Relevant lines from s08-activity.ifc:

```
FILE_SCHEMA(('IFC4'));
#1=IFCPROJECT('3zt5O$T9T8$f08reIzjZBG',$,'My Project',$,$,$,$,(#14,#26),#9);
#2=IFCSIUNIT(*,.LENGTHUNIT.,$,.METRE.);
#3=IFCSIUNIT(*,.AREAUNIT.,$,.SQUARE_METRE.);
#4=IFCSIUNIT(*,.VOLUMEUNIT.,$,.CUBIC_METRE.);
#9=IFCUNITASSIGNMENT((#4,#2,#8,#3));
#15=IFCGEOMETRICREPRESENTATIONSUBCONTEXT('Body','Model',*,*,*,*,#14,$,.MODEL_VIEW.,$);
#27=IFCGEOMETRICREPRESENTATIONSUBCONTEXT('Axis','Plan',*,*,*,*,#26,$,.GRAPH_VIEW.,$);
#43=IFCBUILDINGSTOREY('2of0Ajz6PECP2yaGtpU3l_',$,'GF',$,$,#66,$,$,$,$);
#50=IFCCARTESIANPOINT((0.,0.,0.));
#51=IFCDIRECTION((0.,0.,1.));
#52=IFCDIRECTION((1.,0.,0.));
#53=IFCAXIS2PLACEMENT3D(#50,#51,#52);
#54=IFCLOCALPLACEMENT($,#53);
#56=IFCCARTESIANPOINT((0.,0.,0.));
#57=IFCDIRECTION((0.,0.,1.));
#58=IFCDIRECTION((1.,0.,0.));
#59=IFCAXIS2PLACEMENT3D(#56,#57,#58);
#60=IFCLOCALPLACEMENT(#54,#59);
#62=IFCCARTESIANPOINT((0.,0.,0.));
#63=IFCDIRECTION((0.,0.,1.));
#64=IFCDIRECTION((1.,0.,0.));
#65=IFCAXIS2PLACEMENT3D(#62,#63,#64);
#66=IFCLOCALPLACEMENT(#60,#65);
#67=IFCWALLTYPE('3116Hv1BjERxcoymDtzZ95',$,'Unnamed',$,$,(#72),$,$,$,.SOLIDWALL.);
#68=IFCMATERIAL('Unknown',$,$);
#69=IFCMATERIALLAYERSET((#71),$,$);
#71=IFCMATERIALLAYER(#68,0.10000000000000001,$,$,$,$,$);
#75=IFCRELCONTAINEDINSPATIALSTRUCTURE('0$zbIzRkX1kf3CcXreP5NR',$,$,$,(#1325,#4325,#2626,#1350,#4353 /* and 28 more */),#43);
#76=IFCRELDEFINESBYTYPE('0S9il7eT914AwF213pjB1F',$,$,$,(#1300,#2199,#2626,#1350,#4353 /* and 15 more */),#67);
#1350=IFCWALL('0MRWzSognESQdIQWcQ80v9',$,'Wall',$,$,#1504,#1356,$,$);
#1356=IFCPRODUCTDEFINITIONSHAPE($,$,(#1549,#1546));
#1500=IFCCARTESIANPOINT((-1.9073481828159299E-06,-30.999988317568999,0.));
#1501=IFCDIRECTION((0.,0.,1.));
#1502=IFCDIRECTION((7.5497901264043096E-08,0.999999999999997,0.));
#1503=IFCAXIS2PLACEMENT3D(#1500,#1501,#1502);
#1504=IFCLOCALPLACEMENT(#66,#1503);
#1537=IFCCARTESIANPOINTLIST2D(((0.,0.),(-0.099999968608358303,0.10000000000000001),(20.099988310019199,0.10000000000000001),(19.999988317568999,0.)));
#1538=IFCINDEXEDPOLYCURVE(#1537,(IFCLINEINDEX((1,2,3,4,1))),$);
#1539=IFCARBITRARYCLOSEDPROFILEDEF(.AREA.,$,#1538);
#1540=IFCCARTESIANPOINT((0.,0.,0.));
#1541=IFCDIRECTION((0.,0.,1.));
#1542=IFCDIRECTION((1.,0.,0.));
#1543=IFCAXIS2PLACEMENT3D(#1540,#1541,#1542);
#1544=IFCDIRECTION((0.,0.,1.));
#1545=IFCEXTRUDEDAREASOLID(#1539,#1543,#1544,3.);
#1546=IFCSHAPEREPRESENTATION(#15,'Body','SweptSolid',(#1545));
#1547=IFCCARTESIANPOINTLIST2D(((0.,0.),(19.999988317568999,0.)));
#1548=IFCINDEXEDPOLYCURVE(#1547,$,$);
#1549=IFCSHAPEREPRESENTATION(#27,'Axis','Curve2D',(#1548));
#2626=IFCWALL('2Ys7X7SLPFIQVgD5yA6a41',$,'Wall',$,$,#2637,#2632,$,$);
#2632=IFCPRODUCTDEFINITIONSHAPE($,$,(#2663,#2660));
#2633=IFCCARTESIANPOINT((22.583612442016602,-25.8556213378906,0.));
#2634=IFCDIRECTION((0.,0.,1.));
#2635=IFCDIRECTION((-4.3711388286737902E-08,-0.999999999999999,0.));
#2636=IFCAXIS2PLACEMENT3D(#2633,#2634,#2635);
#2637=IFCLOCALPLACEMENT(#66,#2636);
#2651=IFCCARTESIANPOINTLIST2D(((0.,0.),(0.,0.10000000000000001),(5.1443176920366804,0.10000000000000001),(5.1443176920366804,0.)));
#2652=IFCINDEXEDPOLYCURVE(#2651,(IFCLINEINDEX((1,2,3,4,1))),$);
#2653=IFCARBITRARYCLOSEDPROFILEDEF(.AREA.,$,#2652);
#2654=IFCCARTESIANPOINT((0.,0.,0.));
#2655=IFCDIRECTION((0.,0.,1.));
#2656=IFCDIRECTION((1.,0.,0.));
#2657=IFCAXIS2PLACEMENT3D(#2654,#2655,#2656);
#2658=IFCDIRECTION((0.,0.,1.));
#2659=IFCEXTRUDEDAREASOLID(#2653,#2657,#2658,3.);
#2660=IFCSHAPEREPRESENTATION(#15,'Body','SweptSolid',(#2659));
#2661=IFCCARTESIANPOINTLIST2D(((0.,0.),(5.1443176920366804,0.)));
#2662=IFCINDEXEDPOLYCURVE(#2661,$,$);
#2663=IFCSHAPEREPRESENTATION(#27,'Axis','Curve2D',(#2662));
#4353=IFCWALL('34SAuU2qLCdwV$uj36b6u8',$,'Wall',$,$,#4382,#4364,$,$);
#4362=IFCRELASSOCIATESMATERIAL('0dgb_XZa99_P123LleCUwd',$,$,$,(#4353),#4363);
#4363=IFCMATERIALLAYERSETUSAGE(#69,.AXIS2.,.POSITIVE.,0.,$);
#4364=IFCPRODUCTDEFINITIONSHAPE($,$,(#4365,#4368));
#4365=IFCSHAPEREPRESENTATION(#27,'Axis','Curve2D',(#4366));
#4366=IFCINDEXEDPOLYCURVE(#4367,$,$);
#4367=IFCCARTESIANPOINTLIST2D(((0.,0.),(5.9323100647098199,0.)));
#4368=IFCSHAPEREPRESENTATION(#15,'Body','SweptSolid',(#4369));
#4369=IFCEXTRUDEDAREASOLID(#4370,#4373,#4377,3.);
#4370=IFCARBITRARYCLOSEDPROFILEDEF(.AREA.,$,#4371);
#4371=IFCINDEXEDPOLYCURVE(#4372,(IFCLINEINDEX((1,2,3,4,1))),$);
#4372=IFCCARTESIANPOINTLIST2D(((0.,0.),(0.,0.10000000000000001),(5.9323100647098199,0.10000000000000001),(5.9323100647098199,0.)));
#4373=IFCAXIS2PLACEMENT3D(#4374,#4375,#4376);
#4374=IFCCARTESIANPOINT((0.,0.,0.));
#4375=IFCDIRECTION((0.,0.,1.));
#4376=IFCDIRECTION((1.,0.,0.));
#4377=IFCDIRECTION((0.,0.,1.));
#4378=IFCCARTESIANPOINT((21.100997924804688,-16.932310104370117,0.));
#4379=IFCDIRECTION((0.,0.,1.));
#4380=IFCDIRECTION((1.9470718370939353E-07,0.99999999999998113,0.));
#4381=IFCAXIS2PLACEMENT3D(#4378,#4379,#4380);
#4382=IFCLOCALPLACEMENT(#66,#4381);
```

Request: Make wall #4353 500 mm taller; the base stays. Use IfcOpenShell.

```python
import ifcopenshell
import ifcopenshell.geom
import ifcopenshell.util.representation
import ifcopenshell.util.shape
import ifcopenshell.util.unit

model = ifcopenshell.open("s08-activity.ifc")
unit_scale = ifcopenshell.util.unit.calculate_unit_scale(model)
settings = ifcopenshell.geom.settings()


def volume(element):
    """Net volume in cubic metres, openings subtracted."""
    shape = ifcopenshell.geom.create_shape(settings, element)
    return ifcopenshell.util.shape.get_volume(shape.geometry)


wall = model.by_id(4353)
before = volume(wall)

body = ifcopenshell.util.representation.get_representation(wall, "Model", "Body")
solid = body.Items[0]
old_height = solid.Depth
solid.Depth += 0.5 / unit_scale
after = volume(wall)

print(f"height {old_height:g} -> {solid.Depth:g}, volume {before:.3f} -> {after:.3f} m3")

model.write("s08-activity_v2.ifc")
```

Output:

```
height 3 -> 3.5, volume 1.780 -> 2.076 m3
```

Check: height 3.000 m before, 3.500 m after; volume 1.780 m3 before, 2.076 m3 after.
